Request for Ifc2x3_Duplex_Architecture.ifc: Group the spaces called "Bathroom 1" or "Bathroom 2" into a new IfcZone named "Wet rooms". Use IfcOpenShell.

First a look at what the model holds.

```python
import ifcopenshell

model = ifcopenshell.open("Ifc2x3_Duplex_Architecture.ifc")
print(model.schema)
seen = {}
for space in model.by_type("IfcSpace"):
    seen[space.LongName] = seen.get(space.LongName, 0) + 1
for name, count in sorted(seen.items(), key=str):
    print(count, "x", name)
print("zones:", [z.Name for z in model.by_type("IfcZone")][:20])
```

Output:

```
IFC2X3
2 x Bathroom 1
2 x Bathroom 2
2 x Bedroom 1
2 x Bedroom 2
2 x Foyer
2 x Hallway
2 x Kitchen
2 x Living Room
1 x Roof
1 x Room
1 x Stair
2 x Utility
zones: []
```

```python
import ifcopenshell
import ifcopenshell.api.group
import ifcopenshell.api.root

model = ifcopenshell.open("Ifc2x3_Duplex_Architecture.ifc")

names = {"Bathroom 1", "Bathroom 2"}
spaces = [s for s in model.by_type("IfcSpace") if s.LongName in names]

zone = ifcopenshell.api.root.create_entity(model, ifc_class="IfcZone", name="Wet rooms")
ifcopenshell.api.group.assign_group(model, products=spaces, group=zone)
print(len(spaces), "spaces in", zone.Name)

model.write("Ifc2x3_Duplex_Architecture_v2.ifc")
```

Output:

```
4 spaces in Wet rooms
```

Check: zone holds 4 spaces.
